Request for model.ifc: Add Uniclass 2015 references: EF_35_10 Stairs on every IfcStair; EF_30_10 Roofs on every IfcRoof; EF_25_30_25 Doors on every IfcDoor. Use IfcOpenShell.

First a look at what the model holds.

```python
import ifcopenshell

model = ifcopenshell.open("model.ifc")
print(model.schema)
print("classifications:", [c.Name for c in model.by_type("IfcClassification")])
for ifc_class in ("IfcDoor", "IfcRoof", "IfcStair", "IfcWall", "IfcWindow"):
    print(ifc_class, len(model.by_type(ifc_class)))
```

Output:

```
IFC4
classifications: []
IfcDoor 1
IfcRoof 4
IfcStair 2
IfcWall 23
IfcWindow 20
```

```python
import ifcopenshell
import ifcopenshell.api.classification

model = ifcopenshell.open("model.ifc")

system = ifcopenshell.api.classification.add_classification(model, classification="Uniclass 2015")

codes = {
    "IfcStair": ("EF_35_10", "Stairs"),
    "IfcRoof": ("EF_30_10", "Roofs"),
    "IfcDoor": ("EF_25_30_25", "Doors"),
}
for ifc_class, (code, name) in codes.items():
    products = model.by_type(ifc_class)
    ifcopenshell.api.classification.add_reference(
        model, products=products, classification=system, identification=code, name=name
    )
    print(code, len(products))

model.write("model_edited.ifc")
```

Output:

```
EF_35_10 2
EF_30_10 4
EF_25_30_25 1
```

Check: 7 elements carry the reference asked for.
